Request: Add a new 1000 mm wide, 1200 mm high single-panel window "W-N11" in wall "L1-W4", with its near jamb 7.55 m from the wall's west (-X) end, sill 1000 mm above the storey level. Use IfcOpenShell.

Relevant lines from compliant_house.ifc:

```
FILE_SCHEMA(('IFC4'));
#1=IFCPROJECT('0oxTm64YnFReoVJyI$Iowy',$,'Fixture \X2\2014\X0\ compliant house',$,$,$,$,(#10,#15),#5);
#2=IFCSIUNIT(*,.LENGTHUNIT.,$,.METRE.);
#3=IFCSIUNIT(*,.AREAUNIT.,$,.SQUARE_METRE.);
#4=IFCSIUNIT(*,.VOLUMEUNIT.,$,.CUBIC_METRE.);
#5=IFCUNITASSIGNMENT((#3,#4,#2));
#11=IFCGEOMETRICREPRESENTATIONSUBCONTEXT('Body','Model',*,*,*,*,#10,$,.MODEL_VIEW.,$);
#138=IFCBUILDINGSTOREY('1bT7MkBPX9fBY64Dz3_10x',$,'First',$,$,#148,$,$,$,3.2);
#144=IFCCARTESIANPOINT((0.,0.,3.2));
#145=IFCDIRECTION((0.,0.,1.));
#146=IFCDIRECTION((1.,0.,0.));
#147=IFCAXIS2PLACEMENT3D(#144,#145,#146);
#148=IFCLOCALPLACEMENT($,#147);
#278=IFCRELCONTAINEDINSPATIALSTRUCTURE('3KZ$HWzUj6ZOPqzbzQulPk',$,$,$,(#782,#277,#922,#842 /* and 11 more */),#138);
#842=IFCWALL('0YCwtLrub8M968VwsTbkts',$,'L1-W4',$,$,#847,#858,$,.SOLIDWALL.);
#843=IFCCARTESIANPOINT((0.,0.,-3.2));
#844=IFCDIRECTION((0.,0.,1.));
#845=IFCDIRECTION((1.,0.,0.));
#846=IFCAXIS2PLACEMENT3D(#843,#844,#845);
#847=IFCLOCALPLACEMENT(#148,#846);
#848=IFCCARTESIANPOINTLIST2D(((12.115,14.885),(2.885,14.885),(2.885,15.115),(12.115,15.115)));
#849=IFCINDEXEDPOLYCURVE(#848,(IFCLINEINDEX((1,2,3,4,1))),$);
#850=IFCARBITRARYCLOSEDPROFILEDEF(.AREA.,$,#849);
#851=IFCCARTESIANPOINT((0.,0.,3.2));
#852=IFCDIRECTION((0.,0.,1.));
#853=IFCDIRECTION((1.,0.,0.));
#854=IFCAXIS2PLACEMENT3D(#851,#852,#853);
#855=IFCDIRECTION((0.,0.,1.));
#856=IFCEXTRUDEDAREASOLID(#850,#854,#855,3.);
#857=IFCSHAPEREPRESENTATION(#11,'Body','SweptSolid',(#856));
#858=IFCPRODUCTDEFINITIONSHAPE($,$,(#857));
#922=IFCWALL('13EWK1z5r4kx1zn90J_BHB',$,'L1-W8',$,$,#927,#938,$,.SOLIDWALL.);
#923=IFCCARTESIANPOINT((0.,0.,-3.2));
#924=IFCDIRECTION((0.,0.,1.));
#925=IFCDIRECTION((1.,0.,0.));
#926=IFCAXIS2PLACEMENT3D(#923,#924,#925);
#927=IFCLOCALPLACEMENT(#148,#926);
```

```python
import numpy as np
import ifcopenshell
import ifcopenshell.api.feature
import ifcopenshell.api.geometry
import ifcopenshell.api.root
import ifcopenshell.api.spatial
import ifcopenshell.geom
import ifcopenshell.util.element
import ifcopenshell.util.placement
import ifcopenshell.util.representation
import ifcopenshell.util.shape
import ifcopenshell.util.unit

model = ifcopenshell.open("compliant_house.ifc")
unit_scale = ifcopenshell.util.unit.calculate_unit_scale(model)
settings = ifcopenshell.geom.settings()


def volume(element):
    """Net volume in cubic metres, openings subtracted."""
    shape = ifcopenshell.geom.create_shape(settings, element)
    return ifcopenshell.util.shape.get_volume(shape.geometry)


wall = model.by_guid("0YCwtLrub8M968VwsTbkts")
storey = ifcopenshell.util.element.get_container(wall, ifc_class="IfcBuildingStorey")
context = ifcopenshell.util.representation.get_context(model, "Model", "Body", "MODEL_VIEW")
before = volume(wall)

width, height, from_end, sill = 1, 1.2, 7.55, 1  # metres

# The wall runs along its own X axis, and the end named is its -X end.
wall_shape = ifcopenshell.geom.create_shape(settings, wall)
x, y, z = ifcopenshell.util.shape.get_vertices(wall_shape.geometry).T
start = x.min() + from_end
face, thickness = float(y.min()), float(y.max() - y.min())
wall_matrix = ifcopenshell.util.placement.get_local_placement(wall.ObjectPlacement)
level = ifcopenshell.util.placement.get_local_placement(storey.ObjectPlacement)[2, 3]


def in_wall(x, y):
    """Placement at x, y metres in the wall's axes, at sill height."""
    matrix = wall_matrix.copy()
    matrix[:, 3] = wall_matrix @ np.array([x / unit_scale, y / unit_scale, 0.0, 1.0])
    matrix[2, 3] = level + sill / unit_scale
    return matrix


# Opening: a box that overshoots both wall faces by 50 mm.
opening = ifcopenshell.api.root.create_entity(model, ifc_class="IfcOpeningElement", predefined_type="OPENING")
box = ifcopenshell.api.geometry.add_wall_representation(
    model, context=context, length=width, height=height, thickness=thickness + 0.1
)
ifcopenshell.api.geometry.assign_representation(model, product=opening, representation=box)
ifcopenshell.api.geometry.edit_object_placement(model, product=opening, matrix=in_wall(start, face - 0.05), is_si=False)
ifcopenshell.api.feature.add_feature(model, feature=opening, element=wall)

window = ifcopenshell.api.root.create_entity(model, ifc_class="IfcWindow", name="W-N11", predefined_type="WINDOW")
window.OverallWidth, window.OverallHeight = width / unit_scale, height / unit_scale
window.PartitioningType = "SINGLE_PANEL"
body = ifcopenshell.api.geometry.add_window_representation(
    model,
    context=context,
    overall_width=window.OverallWidth,
    overall_height=window.OverallHeight,
    partition_type="SINGLE_PANEL",
)
ifcopenshell.api.geometry.assign_representation(model, product=window, representation=body)
ifcopenshell.api.spatial.assign_container(model, products=[window], relating_structure=storey)
ifcopenshell.api.feature.add_filling(model, opening=opening, element=window)

# Centre the window in the wall's thickness.
ifcopenshell.api.geometry.edit_object_placement(model, product=window, matrix=in_wall(start, face), is_si=False)
window_shape = ifcopenshell.geom.create_shape(settings, window)
depth = ifcopenshell.util.shape.get_vertices(window_shape.geometry)[:, 1]
offset = face + thickness / 2 - (depth.min() + depth.max()) / 2
ifcopenshell.api.geometry.edit_object_placement(model, product=window, matrix=in_wall(start, offset), is_si=False)

after = volume(wall)

print(f"wall volume {before:.3f} -> {after:.3f} m3")

model.write("compliant_house-out.ifc")
```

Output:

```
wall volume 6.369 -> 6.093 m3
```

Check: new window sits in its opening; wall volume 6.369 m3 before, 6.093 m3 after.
